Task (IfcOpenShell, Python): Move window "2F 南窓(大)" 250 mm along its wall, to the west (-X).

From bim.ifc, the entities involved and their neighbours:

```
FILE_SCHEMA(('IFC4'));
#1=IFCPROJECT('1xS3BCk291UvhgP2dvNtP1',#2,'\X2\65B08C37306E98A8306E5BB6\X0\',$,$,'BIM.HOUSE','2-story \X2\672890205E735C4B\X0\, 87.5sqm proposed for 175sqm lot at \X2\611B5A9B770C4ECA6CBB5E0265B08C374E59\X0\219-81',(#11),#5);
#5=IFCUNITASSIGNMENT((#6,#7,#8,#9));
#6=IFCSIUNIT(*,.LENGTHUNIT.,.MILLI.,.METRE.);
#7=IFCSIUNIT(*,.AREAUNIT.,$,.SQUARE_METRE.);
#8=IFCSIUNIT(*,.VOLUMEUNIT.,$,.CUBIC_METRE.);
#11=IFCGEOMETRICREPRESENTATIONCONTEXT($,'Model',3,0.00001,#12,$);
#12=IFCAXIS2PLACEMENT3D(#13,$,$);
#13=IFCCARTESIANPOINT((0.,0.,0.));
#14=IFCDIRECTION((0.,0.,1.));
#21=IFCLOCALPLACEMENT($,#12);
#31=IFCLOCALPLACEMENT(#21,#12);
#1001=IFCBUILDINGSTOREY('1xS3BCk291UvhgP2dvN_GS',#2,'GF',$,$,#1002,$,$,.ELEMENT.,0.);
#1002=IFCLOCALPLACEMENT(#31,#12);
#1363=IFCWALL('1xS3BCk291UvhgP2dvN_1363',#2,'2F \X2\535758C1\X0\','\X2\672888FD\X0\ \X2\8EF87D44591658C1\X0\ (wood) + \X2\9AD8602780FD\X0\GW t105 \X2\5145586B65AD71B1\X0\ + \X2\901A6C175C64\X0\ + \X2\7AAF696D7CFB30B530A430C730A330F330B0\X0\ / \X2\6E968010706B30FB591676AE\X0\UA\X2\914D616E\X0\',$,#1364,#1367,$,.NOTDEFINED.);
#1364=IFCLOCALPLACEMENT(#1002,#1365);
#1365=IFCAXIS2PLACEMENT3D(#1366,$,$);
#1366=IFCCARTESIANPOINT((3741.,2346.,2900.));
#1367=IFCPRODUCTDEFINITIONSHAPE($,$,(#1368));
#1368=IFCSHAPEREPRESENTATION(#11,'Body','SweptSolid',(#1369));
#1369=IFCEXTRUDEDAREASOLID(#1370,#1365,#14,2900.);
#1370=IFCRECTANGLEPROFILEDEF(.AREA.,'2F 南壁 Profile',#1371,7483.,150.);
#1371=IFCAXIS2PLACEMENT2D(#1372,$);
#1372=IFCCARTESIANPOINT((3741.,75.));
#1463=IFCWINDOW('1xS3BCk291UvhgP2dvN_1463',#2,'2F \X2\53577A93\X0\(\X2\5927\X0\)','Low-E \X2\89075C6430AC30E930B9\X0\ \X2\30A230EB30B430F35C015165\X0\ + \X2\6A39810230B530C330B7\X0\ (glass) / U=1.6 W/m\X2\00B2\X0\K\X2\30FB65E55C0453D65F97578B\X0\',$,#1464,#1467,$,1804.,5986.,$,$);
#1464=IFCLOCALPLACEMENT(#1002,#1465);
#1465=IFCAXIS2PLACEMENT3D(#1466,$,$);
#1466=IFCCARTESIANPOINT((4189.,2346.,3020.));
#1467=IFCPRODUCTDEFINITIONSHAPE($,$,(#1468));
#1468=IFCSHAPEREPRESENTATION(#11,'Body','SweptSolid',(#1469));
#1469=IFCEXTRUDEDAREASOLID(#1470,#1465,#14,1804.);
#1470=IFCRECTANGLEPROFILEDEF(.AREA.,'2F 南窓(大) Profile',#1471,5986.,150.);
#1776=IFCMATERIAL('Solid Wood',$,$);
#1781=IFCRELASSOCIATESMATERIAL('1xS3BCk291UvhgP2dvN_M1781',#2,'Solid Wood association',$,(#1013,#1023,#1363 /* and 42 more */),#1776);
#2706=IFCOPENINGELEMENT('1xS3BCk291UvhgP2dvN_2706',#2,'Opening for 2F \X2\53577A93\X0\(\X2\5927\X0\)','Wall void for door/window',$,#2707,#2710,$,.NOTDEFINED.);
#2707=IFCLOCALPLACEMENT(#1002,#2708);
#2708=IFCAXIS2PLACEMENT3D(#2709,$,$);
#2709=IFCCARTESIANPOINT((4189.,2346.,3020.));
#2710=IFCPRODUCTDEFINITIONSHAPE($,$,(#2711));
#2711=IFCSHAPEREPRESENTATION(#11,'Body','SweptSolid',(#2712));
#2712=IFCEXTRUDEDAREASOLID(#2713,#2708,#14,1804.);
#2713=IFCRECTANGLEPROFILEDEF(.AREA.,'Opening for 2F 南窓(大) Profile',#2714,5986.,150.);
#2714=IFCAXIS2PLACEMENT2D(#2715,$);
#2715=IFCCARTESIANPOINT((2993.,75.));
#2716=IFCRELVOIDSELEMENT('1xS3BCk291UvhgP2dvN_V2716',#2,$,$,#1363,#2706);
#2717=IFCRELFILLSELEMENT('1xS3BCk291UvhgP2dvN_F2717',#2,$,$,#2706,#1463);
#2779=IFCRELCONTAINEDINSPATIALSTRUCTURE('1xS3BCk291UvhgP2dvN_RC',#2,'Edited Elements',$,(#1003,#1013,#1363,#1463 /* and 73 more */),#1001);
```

```python
import ifcopenshell
import ifcopenshell.api.geometry
import ifcopenshell.util.placement
import ifcopenshell.util.unit

model = ifcopenshell.open("bim.ifc")
unit_scale = ifcopenshell.util.unit.calculate_unit_scale(model)

window = model.by_guid("1xS3BCk291UvhgP2dvN_1463")
opening = window.FillsVoids[0].RelatingOpeningElement
wall = opening.VoidsElements[0].RelatingBuildingElement

wall_matrix = ifcopenshell.util.placement.get_local_placement(wall.ObjectPlacement)
shift = wall_matrix[:3, 0] * -0.25 / unit_scale
before = ifcopenshell.util.placement.get_local_placement(window.ObjectPlacement)[:3, 3].copy()

# The window is not placed relative to its opening, so move both.
for product in (opening, window):
    matrix = ifcopenshell.util.placement.get_local_placement(product.ObjectPlacement)
    matrix[:3, 3] += shift
    ifcopenshell.api.geometry.edit_object_placement(model, product=product, matrix=matrix, is_si=False)

after = ifcopenshell.util.placement.get_local_placement(window.ObjectPlacement)[:3, 3]
print("window moved by", (after - before).round(3) + 0.0)

model.write("bim_rev.ifc")
```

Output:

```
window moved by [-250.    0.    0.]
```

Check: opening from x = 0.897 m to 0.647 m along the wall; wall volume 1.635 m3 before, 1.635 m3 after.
